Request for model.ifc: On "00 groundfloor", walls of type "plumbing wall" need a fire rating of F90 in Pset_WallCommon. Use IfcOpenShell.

First a look at what the model holds.

```python
import ifcopenshell
import ifcopenshell.util.element

model = ifcopenshell.open("model.ifc")
print(model.schema)
storey = next(s for s in model.by_type("IfcBuildingStorey") if s.Name == "00 groundfloor")
walls = [e for e in ifcopenshell.util.element.get_decomposition(storey) if e.is_a("IfcWall")]
seen = {}
for e in walls:
    element_type = ifcopenshell.util.element.get_type(e)
    key = (element_type.Name if element_type != e and element_type else None, ifcopenshell.util.element.get_pset(e, "Pset_WallCommon", "FireRating"))
    seen[key] = seen.get(key, 0) + 1
for (name, value), count in sorted(seen.items(), key=str):
    print(count, "x", name, "|", value)
```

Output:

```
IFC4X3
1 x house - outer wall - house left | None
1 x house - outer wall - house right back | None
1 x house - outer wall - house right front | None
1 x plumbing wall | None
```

```python
import ifcopenshell
import ifcopenshell.api.pset
import ifcopenshell.util.element

model = ifcopenshell.open("model.ifc")

storey = next(s for s in model.by_type("IfcBuildingStorey") if s.Name == "00 groundfloor")
walls = [e for e in ifcopenshell.util.element.get_decomposition(storey) if e.is_a("IfcWall")]

count = 0
for e in walls:
    element_type = ifcopenshell.util.element.get_type(e)
    if element_type in (None, e) or element_type.Name != "plumbing wall":
        continue
    # add_pset returns the element's existing set when there is one.
    pset = ifcopenshell.api.pset.add_pset(model, product=e, name="Pset_WallCommon")
    ifcopenshell.api.pset.edit_pset(model, pset=pset, properties={"FireRating": "F90"})
    count += 1

print(count, "walls updated")

model.write("model_updated.ifc")
```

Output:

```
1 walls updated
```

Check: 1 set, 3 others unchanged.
